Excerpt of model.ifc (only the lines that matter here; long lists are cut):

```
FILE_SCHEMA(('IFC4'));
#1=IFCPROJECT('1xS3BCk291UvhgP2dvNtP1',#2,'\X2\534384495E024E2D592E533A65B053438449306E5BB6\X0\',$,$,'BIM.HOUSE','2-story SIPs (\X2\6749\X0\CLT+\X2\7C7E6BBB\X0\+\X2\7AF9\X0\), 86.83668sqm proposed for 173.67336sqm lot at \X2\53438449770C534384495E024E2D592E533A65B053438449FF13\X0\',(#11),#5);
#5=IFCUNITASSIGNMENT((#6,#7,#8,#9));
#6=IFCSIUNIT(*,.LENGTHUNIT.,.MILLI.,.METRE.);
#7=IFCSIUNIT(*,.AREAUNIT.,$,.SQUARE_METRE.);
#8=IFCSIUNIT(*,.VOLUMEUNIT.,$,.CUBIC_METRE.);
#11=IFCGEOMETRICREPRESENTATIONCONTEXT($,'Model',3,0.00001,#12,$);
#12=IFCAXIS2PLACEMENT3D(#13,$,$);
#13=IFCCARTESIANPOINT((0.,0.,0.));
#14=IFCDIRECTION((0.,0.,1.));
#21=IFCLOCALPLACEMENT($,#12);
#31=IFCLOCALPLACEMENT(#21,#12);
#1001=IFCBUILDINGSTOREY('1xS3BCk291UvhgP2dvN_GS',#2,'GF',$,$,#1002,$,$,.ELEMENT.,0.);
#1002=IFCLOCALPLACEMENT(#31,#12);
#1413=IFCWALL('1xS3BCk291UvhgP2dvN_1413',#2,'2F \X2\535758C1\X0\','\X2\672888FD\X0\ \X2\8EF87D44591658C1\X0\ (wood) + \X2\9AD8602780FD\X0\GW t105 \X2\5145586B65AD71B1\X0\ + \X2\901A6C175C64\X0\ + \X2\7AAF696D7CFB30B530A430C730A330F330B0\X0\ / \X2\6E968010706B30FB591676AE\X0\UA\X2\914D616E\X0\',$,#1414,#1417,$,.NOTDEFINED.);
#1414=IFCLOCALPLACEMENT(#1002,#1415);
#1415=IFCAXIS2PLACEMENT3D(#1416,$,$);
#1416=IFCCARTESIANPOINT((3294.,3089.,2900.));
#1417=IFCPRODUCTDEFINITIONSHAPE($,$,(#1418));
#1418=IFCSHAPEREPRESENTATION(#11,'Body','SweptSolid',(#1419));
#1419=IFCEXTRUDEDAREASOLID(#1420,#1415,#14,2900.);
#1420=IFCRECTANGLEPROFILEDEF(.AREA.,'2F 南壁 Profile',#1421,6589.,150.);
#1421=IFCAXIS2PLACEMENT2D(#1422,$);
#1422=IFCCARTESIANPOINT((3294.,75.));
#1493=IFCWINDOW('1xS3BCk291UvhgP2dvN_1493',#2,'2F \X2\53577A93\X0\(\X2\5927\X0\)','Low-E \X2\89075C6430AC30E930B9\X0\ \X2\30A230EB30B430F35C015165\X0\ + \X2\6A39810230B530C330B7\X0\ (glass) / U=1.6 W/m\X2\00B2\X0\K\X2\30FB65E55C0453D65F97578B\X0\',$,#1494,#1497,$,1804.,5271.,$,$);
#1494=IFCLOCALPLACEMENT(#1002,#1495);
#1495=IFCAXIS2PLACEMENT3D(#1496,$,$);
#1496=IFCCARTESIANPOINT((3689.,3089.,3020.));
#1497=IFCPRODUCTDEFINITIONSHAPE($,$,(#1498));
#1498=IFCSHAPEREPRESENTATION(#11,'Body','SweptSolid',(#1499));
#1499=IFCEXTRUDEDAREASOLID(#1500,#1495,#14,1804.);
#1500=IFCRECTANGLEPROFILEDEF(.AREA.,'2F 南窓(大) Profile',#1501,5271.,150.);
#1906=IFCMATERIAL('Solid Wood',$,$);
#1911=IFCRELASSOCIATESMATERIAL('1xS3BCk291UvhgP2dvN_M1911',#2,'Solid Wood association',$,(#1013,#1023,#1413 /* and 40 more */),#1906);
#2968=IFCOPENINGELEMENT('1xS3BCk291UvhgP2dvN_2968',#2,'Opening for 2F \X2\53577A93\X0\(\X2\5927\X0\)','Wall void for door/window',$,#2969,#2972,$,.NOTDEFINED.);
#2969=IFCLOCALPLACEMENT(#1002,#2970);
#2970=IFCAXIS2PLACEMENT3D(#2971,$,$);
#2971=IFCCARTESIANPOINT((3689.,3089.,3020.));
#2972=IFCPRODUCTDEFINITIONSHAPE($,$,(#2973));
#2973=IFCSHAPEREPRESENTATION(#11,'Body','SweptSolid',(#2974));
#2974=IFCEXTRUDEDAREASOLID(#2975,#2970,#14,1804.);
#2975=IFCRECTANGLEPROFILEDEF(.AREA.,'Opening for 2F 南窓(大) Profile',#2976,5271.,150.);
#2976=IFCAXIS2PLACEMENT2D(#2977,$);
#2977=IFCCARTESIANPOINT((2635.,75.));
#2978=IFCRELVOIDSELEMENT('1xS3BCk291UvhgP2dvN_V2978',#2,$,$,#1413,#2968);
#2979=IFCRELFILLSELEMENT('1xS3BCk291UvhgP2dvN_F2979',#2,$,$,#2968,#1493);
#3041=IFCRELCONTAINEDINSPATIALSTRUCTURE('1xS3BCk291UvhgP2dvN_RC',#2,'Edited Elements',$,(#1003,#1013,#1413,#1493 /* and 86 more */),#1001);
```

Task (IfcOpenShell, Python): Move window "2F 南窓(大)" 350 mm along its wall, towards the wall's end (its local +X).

```python
import ifcopenshell
import ifcopenshell.api.geometry
import ifcopenshell.util.placement
import ifcopenshell.util.unit

model = ifcopenshell.open("model.ifc")
unit_scale = ifcopenshell.util.unit.calculate_unit_scale(model)

window = model.by_id(1493)
opening = window.FillsVoids[0].RelatingOpeningElement
wall = opening.VoidsElements[0].RelatingBuildingElement

wall_matrix = ifcopenshell.util.placement.get_local_placement(wall.ObjectPlacement)
shift = wall_matrix[:3, 0] * 0.35 / unit_scale
before = ifcopenshell.util.placement.get_local_placement(window.ObjectPlacement)[:3, 3].copy()

# The window is not placed relative to its opening, so move both.
for product in (opening, window):
    matrix = ifcopenshell.util.placement.get_local_placement(product.ObjectPlacement)
    matrix[:3, 3] += shift
    ifcopenshell.api.geometry.edit_object_placement(model, product=product, matrix=matrix, is_si=False)

after = ifcopenshell.util.placement.get_local_placement(window.ObjectPlacement)[:3, 3]
print("window moved by", (after - before).round(3) + 0.0)

model.write("model_updated.ifc")
```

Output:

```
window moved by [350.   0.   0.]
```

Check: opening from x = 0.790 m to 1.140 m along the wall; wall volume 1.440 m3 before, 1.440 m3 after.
